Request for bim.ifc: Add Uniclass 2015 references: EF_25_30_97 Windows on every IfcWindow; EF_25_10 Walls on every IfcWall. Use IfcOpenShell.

First a look at what the model holds.

```python
import ifcopenshell

model = ifcopenshell.open("bim.ifc")
print(model.schema)
print("classifications:", [c.Name for c in model.by_type("IfcClassification")])
for ifc_class in ("IfcDoor", "IfcRoof", "IfcStair", "IfcWall", "IfcWindow"):
    print(ifc_class, len(model.by_type(ifc_class)))
```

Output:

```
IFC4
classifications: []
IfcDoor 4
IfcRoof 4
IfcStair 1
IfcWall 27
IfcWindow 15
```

```python
import ifcopenshell
import ifcopenshell.api.classification

model = ifcopenshell.open("bim.ifc")

system = ifcopenshell.api.classification.add_classification(model, classification="Uniclass 2015")

codes = {
    "IfcWindow": ("EF_25_30_97", "Windows"),
    "IfcWall": ("EF_25_10", "Walls"),
}
for ifc_class, (code, name) in codes.items():
    products = model.by_type(ifc_class)
    ifcopenshell.api.classification.add_reference(
        model, products=products, classification=system, identification=code, name=name
    )
    print(code, len(products))

model.write("bim_updated.ifc")
```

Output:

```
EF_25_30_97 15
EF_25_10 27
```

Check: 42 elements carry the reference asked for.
